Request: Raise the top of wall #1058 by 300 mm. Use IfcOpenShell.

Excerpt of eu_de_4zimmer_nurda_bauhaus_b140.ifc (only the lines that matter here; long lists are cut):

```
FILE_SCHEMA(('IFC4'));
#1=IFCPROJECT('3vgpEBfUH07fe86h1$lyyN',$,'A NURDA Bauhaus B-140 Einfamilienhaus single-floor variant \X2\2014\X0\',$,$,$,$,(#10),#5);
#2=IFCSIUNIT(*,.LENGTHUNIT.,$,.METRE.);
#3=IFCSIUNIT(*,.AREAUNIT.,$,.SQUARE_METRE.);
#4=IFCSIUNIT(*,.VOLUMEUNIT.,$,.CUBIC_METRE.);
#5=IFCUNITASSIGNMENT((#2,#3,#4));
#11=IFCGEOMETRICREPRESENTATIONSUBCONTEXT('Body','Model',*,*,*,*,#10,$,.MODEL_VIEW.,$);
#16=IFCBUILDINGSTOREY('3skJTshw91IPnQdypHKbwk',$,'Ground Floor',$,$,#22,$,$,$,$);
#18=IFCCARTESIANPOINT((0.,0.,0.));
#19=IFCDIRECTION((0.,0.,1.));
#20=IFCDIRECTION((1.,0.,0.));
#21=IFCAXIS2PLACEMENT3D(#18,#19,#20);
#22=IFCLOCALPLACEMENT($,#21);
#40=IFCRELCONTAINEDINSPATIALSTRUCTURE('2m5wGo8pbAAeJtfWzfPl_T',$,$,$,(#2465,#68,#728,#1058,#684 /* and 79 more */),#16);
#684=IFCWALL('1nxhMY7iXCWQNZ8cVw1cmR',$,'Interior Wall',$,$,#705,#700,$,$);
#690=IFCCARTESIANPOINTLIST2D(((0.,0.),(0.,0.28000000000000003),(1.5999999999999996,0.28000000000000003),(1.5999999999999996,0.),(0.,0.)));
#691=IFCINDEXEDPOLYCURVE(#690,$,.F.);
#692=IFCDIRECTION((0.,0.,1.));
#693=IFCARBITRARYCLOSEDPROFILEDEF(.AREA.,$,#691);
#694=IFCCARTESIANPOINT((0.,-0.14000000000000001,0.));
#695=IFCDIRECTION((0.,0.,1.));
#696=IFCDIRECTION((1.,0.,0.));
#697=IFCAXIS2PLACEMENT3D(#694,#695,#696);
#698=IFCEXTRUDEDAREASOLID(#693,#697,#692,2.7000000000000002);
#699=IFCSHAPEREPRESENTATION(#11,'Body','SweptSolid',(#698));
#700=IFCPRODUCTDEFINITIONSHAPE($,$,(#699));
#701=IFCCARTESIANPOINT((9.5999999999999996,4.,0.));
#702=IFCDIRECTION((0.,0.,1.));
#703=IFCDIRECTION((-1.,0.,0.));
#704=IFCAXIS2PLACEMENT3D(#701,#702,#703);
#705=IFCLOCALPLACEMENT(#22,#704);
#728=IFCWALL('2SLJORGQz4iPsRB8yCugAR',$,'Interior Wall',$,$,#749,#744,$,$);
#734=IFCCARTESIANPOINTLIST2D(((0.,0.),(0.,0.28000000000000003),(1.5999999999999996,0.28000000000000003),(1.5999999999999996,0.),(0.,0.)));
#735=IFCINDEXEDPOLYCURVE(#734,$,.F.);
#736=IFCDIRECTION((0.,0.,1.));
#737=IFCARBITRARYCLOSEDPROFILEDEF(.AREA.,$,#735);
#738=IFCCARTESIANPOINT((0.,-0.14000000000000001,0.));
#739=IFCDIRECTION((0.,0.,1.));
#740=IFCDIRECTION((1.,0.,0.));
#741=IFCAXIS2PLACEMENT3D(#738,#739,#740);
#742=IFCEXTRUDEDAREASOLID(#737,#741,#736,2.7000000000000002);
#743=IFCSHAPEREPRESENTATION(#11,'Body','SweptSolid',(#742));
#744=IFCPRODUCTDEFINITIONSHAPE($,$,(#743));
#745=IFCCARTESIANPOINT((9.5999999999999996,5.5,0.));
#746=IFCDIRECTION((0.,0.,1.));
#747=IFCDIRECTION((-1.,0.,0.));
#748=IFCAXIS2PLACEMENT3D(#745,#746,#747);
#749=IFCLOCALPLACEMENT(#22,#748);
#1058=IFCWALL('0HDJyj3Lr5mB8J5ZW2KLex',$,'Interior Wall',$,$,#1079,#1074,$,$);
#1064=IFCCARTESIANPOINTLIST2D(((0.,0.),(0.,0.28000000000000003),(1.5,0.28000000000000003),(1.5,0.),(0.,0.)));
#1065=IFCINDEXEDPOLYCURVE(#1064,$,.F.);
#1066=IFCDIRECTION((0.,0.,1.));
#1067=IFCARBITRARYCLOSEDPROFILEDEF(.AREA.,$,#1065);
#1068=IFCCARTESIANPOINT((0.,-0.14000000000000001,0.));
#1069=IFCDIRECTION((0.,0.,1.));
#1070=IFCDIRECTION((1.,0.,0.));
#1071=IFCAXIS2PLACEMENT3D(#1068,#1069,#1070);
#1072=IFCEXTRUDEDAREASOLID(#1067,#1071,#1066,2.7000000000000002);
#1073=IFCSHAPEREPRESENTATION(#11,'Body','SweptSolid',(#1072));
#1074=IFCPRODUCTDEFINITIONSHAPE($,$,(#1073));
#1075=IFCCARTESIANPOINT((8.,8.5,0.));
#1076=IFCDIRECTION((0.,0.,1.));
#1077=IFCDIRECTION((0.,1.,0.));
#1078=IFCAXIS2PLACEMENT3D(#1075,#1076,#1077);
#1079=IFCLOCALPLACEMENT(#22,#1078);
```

```python
import ifcopenshell
import ifcopenshell.geom
import ifcopenshell.util.representation
import ifcopenshell.util.shape

model = ifcopenshell.open("eu_de_4zimmer_nurda_bauhaus_b140.ifc")
settings = ifcopenshell.geom.settings()


def volume(element):
    """Net volume in cubic metres, openings subtracted."""
    shape = ifcopenshell.geom.create_shape(settings, element)
    return ifcopenshell.util.shape.get_volume(shape.geometry)


wall = model.by_guid("0HDJyj3Lr5mB8J5ZW2KLex")
before = volume(wall)

body = ifcopenshell.util.representation.get_representation(wall, "Model", "Body")
solid = body.Items[0]
old_height = solid.Depth
solid.Depth += 0.3
after = volume(wall)

print(f"height {old_height:g} -> {solid.Depth:g}, volume {before:.3f} -> {after:.3f} m3")

model.write("eu_de_4zimmer_nurda_bauhaus_b140_rev.ifc")
```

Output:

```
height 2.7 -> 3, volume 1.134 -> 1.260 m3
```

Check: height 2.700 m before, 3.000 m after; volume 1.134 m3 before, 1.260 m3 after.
